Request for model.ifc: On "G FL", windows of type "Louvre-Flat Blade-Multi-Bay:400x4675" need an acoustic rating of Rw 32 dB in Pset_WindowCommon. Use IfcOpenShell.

First a look at what the model holds.

```python
import ifcopenshell
import ifcopenshell.util.element

model = ifcopenshell.open("model.ifc")
print(model.schema)
storey = next(s for s in model.by_type("IfcBuildingStorey") if s.Name == "G FL")
windows = [e for e in ifcopenshell.util.element.get_decomposition(storey) if e.is_a("IfcWindow")]
seen = {}
for e in windows:
    element_type = ifcopenshell.util.element.get_type(e)
    key = (element_type.Name if element_type != e and element_type else None, ifcopenshell.util.element.get_pset(e, "Pset_WindowCommon", "AcousticRating"))
    seen[key] = seen.get(key, 0) + 1
for (name, value), count in sorted(seen.items(), key=str):
    print(count, "x", name, "|", value)
```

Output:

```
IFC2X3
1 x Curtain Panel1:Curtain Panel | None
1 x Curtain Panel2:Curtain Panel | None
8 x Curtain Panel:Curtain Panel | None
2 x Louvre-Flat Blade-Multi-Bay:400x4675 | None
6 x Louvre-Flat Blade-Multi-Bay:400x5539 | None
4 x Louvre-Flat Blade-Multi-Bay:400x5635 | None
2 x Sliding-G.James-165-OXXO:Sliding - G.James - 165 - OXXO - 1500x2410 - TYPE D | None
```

```python
import ifcopenshell
import ifcopenshell.api.pset
import ifcopenshell.util.element

model = ifcopenshell.open("model.ifc")

storey = next(s for s in model.by_type("IfcBuildingStorey") if s.Name == "G FL")
windows = [e for e in ifcopenshell.util.element.get_decomposition(storey) if e.is_a("IfcWindow")]

count = 0
for e in windows:
    element_type = ifcopenshell.util.element.get_type(e)
    if element_type in (None, e) or element_type.Name != "Louvre-Flat Blade-Multi-Bay:400x4675":
        continue
    # add_pset returns the element's existing set when there is one.
    pset = ifcopenshell.api.pset.add_pset(model, product=e, name="Pset_WindowCommon")
    ifcopenshell.api.pset.edit_pset(model, pset=pset, properties={"AcousticRating": "Rw 32 dB"})
    count += 1

print(count, "windows updated")

model.write("model_v2.ifc")
```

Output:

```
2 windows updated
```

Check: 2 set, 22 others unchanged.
